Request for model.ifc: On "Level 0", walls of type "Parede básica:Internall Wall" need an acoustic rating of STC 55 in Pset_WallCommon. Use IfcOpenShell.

First a look at what the model holds.

```python
import ifcopenshell
import ifcopenshell.util.element

model = ifcopenshell.open("model.ifc")
print(model.schema)
storey = next(s for s in model.by_type("IfcBuildingStorey") if s.Name == "Level 0")
walls = [e for e in ifcopenshell.util.element.get_decomposition(storey) if e.is_a("IfcWall")]
seen = {}
for e in walls:
    element_type = ifcopenshell.util.element.get_type(e)
    key = (element_type.Name if element_type != e and element_type else None, ifcopenshell.util.element.get_pset(e, "Pset_WallCommon", "AcousticRating"))
    seen[key] = seen.get(key, 0) + 1
for (name, value), count in sorted(seen.items(), key=str):
    print(count, "x", name, "|", value)
```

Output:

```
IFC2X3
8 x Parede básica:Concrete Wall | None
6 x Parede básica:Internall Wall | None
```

```python
import ifcopenshell
import ifcopenshell.api.pset
import ifcopenshell.util.element

model = ifcopenshell.open("model.ifc")

storey = next(s for s in model.by_type("IfcBuildingStorey") if s.Name == "Level 0")
walls = [e for e in ifcopenshell.util.element.get_decomposition(storey) if e.is_a("IfcWall")]

count = 0
for e in walls:
    element_type = ifcopenshell.util.element.get_type(e)
    if element_type in (None, e) or element_type.Name != "Parede básica:Internall Wall":
        continue
    # add_pset returns the element's existing set when there is one.
    pset = ifcopenshell.api.pset.add_pset(model, product=e, name="Pset_WallCommon")
    ifcopenshell.api.pset.edit_pset(model, pset=pset, properties={"AcousticRating": "STC 55"})
    count += 1

print(count, "walls updated")

model.write("model-out.ifc")
```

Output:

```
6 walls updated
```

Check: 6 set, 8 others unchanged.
